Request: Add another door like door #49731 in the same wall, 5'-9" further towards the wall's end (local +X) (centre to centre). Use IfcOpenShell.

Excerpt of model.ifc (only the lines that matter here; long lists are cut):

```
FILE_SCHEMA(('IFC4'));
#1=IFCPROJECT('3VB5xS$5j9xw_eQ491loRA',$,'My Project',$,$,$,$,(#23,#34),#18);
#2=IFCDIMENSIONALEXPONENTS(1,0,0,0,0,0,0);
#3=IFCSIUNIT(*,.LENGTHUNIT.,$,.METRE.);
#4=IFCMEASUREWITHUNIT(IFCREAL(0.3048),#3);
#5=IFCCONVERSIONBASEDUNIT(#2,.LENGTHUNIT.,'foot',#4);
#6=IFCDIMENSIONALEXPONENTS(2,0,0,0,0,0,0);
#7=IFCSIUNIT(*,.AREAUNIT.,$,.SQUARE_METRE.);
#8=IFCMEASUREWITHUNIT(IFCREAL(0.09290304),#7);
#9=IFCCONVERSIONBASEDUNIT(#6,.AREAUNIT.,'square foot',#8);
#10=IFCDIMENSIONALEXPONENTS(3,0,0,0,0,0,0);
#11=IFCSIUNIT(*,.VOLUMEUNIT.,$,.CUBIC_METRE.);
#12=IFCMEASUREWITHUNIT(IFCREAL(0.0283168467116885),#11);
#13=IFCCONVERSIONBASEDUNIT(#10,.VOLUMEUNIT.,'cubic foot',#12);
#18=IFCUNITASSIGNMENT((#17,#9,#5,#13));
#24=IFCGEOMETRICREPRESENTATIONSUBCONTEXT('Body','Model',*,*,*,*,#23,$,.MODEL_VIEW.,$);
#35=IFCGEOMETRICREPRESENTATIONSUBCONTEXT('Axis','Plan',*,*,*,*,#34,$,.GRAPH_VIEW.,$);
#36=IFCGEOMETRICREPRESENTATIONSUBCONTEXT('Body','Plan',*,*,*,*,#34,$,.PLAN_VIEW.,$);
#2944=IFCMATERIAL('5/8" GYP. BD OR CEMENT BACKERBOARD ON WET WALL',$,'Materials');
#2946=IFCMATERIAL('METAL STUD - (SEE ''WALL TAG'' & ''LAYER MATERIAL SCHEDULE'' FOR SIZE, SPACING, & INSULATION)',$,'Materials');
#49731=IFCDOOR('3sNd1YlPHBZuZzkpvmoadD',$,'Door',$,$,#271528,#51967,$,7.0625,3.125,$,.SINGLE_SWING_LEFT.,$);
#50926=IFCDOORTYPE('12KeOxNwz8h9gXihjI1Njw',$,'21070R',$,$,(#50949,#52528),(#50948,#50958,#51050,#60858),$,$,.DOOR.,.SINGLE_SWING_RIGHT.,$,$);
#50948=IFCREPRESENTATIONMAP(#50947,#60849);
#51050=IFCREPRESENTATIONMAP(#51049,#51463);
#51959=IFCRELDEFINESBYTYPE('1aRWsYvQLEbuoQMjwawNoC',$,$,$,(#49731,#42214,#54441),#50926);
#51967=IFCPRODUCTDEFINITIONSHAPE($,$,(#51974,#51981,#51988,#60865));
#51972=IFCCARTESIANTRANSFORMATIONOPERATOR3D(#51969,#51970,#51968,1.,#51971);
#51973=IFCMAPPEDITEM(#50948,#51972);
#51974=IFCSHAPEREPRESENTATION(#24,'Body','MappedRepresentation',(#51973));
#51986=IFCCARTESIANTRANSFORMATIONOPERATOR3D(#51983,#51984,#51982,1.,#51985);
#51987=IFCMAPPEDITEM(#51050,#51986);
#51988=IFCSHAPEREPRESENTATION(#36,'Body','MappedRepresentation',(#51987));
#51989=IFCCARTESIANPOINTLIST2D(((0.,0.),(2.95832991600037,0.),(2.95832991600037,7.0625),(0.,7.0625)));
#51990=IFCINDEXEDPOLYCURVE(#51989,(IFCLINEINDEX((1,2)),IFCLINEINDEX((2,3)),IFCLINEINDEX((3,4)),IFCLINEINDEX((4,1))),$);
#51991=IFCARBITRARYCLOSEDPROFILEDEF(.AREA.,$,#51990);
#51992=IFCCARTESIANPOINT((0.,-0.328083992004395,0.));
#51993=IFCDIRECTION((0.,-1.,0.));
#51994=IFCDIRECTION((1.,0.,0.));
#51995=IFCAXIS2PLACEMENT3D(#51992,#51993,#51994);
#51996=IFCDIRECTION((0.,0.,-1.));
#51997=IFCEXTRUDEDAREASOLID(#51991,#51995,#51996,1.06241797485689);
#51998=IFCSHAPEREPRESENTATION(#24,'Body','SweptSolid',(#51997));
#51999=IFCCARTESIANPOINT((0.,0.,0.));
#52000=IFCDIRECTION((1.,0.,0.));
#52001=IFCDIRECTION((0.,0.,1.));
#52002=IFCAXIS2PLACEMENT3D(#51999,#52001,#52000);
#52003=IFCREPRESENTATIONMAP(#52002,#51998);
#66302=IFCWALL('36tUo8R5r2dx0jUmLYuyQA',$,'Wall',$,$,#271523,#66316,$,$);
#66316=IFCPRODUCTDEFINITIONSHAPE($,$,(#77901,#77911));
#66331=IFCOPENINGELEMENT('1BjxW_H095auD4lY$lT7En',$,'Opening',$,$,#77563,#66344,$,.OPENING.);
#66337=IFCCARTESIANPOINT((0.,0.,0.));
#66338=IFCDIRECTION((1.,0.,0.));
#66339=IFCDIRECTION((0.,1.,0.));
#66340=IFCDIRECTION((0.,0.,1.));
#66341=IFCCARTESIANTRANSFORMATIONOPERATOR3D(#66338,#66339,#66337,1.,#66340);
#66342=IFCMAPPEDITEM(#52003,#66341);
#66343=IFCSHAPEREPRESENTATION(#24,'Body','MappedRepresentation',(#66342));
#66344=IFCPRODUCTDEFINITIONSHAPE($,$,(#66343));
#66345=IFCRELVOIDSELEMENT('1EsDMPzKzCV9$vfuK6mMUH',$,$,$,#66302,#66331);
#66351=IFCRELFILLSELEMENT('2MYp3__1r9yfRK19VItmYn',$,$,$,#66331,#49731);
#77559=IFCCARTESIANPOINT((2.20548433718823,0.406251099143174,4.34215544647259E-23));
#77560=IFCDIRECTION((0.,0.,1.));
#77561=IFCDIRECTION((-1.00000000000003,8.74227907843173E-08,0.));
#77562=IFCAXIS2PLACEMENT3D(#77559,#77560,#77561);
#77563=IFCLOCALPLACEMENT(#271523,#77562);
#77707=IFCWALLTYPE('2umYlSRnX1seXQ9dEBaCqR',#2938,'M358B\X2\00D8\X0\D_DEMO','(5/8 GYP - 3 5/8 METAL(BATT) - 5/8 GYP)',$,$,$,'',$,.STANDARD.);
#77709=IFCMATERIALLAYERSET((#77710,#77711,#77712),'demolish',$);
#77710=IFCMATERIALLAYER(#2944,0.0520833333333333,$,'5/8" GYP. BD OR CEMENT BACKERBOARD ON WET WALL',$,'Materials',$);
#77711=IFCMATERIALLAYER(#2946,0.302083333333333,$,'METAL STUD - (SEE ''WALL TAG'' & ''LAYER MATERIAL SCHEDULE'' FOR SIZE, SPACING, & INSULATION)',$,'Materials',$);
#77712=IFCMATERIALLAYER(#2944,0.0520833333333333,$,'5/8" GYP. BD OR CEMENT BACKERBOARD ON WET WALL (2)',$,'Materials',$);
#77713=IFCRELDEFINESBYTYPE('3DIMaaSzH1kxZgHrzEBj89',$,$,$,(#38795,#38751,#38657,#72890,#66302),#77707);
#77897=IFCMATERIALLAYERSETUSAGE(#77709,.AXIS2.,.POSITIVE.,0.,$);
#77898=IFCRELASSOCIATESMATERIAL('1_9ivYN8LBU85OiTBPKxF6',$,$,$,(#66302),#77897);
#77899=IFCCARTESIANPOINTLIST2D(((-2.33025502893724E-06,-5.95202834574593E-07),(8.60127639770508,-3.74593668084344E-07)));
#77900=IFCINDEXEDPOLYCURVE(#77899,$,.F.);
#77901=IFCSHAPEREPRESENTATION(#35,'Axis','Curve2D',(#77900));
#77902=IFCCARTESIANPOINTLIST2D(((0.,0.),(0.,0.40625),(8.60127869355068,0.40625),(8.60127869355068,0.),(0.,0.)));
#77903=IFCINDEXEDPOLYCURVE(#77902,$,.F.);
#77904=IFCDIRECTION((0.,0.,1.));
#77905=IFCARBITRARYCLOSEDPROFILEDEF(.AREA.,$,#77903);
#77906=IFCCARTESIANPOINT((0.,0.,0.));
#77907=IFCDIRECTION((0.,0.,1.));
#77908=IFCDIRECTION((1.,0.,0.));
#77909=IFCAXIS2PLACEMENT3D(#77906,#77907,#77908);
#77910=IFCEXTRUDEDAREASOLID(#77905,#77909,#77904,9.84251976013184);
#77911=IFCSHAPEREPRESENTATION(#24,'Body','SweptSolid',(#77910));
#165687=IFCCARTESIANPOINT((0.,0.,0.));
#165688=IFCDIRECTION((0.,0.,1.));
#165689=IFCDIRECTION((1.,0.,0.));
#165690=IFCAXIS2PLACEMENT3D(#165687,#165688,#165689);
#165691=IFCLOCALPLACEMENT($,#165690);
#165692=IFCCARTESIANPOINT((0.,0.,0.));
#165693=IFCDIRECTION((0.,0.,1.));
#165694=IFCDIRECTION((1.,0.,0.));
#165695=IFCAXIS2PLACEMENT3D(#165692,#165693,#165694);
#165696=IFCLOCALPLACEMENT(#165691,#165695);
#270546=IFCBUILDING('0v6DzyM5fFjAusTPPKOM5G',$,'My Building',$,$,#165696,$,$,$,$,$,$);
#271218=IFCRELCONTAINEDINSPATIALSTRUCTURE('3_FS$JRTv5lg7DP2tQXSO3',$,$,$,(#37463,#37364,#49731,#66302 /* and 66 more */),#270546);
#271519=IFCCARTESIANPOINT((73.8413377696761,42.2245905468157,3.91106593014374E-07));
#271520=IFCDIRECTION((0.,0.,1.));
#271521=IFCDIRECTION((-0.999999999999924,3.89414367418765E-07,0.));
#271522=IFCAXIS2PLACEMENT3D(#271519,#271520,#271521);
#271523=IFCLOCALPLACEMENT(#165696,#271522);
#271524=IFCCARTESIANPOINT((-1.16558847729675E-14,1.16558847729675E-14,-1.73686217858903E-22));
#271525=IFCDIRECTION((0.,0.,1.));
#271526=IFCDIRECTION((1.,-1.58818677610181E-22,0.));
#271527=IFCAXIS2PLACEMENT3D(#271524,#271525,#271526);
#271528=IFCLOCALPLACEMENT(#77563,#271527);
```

```python
import ifcopenshell
import ifcopenshell.api.feature
import ifcopenshell.api.geometry
import ifcopenshell.api.root
import ifcopenshell.geom
import ifcopenshell.util.element
import ifcopenshell.util.placement
import ifcopenshell.util.shape
import ifcopenshell.util.unit

model = ifcopenshell.open("model.ifc")
unit_scale = ifcopenshell.util.unit.calculate_unit_scale(model)
settings = ifcopenshell.geom.settings()


def volume(element):
    """Net volume in cubic metres, openings subtracted."""
    shape = ifcopenshell.geom.create_shape(settings, element)
    return ifcopenshell.util.shape.get_volume(shape.geometry)


door = model.by_id(49731)
opening = door.FillsVoids[0].RelatingOpeningElement
wall = opening.VoidsElements[0].RelatingBuildingElement
before = volume(wall)
shift = ifcopenshell.util.placement.get_local_placement(wall.ObjectPlacement)[:3, 0] * 69 * 0.0254 / unit_scale

# copy_class copies the void relationship, type, container and properties, but no geometry.
new_opening = ifcopenshell.api.root.copy_class(model, product=opening)
new_opening.Representation = ifcopenshell.util.element.copy_deep(
    model, opening.Representation, exclude=["IfcGeometricRepresentationContext", "IfcRepresentationMap"]
)
new_door = ifcopenshell.api.root.copy_class(model, product=door)
new_door.Representation = ifcopenshell.util.element.copy_deep(
    model, door.Representation, exclude=["IfcGeometricRepresentationContext", "IfcRepresentationMap"]
)
ifcopenshell.api.feature.add_filling(model, opening=new_opening, element=new_door)

for old, new in ((opening, new_opening), (door, new_door)):
    matrix = ifcopenshell.util.placement.get_local_placement(old.ObjectPlacement)
    matrix[:3, 3] += shift
    ifcopenshell.api.geometry.edit_object_placement(model, product=new, matrix=matrix, is_si=False)

after = volume(wall)

print(f"wall volume {before:.3f} -> {after:.3f} m3")

model.write("model_edited.ifc")
```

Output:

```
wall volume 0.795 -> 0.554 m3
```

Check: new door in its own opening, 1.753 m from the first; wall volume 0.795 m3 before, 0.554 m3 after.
